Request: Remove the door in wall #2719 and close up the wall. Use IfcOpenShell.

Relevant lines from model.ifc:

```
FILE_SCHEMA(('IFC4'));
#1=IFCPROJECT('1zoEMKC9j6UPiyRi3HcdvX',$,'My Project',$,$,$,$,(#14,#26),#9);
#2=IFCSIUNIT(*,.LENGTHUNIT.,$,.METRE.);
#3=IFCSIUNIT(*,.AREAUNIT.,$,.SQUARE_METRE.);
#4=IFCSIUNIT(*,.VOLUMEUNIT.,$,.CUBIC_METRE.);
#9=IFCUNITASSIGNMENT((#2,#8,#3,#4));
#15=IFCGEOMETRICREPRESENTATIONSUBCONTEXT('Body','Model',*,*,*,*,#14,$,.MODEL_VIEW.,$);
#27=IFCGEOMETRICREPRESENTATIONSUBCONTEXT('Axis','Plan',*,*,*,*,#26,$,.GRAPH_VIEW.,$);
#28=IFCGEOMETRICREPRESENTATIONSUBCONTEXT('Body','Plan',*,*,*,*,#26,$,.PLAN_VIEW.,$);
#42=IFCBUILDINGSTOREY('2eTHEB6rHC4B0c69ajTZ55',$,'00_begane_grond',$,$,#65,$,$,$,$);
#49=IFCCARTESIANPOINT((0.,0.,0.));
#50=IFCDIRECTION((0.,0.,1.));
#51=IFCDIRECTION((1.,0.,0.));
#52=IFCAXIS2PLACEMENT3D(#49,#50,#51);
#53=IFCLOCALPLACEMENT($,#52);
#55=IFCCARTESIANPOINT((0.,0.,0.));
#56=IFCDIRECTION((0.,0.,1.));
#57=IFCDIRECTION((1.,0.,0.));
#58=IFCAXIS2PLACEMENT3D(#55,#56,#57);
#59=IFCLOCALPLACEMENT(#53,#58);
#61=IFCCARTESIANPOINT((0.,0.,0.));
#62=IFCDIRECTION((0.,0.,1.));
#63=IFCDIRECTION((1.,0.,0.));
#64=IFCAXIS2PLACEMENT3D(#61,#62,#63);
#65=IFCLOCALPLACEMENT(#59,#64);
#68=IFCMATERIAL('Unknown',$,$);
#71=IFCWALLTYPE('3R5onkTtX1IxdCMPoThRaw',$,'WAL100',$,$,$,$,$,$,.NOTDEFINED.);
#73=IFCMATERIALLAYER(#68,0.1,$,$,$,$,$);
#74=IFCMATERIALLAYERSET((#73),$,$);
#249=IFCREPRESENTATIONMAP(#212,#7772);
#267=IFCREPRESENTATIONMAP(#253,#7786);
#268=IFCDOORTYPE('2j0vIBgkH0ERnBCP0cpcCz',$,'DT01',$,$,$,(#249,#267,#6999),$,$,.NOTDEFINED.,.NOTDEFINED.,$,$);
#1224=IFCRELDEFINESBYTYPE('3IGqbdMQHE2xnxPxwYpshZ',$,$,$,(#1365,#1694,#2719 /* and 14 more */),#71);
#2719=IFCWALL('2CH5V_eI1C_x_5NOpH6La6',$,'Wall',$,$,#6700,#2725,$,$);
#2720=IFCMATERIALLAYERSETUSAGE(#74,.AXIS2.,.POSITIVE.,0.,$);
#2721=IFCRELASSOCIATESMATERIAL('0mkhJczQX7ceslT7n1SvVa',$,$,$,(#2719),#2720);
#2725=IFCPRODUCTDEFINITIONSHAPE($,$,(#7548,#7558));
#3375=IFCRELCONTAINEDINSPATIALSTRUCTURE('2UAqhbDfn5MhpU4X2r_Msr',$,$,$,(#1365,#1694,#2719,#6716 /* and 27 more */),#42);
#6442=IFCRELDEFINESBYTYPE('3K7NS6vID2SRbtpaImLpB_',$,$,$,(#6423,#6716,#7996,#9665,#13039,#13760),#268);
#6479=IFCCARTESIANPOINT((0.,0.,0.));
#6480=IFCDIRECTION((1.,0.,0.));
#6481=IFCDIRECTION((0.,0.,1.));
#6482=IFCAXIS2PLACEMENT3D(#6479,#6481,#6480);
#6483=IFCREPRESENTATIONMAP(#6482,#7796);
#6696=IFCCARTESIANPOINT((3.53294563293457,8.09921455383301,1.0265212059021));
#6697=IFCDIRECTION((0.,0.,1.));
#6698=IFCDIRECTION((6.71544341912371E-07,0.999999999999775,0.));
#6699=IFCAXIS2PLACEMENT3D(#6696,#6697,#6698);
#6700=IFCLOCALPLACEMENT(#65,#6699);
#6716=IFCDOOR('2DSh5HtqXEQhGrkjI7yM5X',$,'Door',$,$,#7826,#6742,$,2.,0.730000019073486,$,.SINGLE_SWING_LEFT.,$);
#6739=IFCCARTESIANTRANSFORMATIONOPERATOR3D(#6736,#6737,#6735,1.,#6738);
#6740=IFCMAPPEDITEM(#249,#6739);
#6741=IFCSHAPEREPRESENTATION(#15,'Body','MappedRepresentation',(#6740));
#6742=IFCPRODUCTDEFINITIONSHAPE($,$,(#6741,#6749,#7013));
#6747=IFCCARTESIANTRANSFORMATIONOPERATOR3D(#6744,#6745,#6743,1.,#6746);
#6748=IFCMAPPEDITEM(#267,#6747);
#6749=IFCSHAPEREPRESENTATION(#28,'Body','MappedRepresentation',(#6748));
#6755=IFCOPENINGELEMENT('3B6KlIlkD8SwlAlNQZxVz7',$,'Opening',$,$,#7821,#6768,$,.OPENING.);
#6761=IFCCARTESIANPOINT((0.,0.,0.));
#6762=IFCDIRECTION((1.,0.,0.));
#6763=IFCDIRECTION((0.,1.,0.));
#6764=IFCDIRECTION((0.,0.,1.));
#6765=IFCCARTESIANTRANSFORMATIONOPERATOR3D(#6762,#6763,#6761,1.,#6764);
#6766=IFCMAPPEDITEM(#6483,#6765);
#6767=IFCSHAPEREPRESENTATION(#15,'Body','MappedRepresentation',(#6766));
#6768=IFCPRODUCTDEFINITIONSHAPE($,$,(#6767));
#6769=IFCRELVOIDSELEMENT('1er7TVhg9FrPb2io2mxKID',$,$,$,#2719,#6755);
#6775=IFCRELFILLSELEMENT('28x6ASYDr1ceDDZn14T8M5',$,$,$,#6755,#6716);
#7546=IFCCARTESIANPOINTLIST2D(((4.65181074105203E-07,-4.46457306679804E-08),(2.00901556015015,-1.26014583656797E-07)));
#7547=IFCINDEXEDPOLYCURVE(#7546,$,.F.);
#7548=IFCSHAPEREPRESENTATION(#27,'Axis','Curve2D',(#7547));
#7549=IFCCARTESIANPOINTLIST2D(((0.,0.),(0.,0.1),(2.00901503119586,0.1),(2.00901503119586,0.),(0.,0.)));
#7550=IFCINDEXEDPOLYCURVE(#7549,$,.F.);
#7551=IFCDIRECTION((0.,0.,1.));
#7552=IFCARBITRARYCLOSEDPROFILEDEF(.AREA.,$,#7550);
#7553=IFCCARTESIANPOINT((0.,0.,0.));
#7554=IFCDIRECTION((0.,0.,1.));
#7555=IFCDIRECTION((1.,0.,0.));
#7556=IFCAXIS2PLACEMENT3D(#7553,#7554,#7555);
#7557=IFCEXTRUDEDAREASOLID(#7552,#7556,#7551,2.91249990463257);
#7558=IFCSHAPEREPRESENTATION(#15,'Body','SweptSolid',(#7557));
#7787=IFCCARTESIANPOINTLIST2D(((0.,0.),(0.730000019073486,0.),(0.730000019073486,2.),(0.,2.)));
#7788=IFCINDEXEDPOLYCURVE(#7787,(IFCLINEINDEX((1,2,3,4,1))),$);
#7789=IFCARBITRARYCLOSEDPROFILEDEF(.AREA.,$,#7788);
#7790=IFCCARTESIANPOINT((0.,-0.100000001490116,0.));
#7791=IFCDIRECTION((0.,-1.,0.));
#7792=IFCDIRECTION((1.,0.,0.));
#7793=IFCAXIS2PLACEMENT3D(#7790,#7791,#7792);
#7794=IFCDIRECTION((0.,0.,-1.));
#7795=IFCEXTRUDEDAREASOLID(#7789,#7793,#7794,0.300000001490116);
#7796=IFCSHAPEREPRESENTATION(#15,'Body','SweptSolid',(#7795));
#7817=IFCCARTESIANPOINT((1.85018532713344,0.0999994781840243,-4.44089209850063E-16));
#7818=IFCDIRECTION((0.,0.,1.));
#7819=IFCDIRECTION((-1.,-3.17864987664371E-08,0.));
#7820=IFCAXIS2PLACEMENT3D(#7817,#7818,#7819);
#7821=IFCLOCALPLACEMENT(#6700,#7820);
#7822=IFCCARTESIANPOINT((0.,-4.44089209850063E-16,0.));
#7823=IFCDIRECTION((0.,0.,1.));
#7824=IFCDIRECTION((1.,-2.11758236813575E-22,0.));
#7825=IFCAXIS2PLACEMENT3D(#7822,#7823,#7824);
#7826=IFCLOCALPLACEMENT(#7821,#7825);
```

```python
import ifcopenshell
import ifcopenshell.api.feature
import ifcopenshell.api.root
import ifcopenshell.geom
import ifcopenshell.util.shape

model = ifcopenshell.open("model.ifc")
settings = ifcopenshell.geom.settings()


def volume(element):
    """Net volume in cubic metres, openings subtracted."""
    shape = ifcopenshell.geom.create_shape(settings, element)
    return ifcopenshell.util.shape.get_volume(shape.geometry)


door = model.by_id(6716)
opening = door.FillsVoids[0].RelatingOpeningElement
wall = opening.VoidsElements[0].RelatingBuildingElement
before = volume(wall)

ifcopenshell.api.root.remove_product(model, product=door)
ifcopenshell.api.feature.remove_feature(model, feature=opening)

after = volume(wall)

print(f"wall volume {before:.3f} -> {after:.3f} m3")

model.write("model_updated.ifc")
```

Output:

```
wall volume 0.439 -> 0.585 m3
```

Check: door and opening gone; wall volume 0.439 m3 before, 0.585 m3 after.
